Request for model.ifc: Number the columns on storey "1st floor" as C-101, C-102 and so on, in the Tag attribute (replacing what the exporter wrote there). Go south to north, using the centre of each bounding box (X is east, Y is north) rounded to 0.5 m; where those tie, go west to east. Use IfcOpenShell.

First a look at what the model holds.

```python
import ifcopenshell
import ifcopenshell.util.element
import ifcopenshell.util.placement

model = ifcopenshell.open("model.ifc")
print(model.schema)
storey = next(s for s in model.by_type("IfcBuildingStorey") if s.Name == "1st floor")
columns = [e for e in ifcopenshell.util.element.get_decomposition(storey) if e.is_a("IfcColumn")]
for e in sorted(columns, key=lambda e: e.id()):
    origin = ifcopenshell.util.placement.get_local_placement(e.ObjectPlacement)[:3, 3]
    print(e.id(), e.Tag, e.Name, origin.round(2) + 0.0, sep=" | ")
```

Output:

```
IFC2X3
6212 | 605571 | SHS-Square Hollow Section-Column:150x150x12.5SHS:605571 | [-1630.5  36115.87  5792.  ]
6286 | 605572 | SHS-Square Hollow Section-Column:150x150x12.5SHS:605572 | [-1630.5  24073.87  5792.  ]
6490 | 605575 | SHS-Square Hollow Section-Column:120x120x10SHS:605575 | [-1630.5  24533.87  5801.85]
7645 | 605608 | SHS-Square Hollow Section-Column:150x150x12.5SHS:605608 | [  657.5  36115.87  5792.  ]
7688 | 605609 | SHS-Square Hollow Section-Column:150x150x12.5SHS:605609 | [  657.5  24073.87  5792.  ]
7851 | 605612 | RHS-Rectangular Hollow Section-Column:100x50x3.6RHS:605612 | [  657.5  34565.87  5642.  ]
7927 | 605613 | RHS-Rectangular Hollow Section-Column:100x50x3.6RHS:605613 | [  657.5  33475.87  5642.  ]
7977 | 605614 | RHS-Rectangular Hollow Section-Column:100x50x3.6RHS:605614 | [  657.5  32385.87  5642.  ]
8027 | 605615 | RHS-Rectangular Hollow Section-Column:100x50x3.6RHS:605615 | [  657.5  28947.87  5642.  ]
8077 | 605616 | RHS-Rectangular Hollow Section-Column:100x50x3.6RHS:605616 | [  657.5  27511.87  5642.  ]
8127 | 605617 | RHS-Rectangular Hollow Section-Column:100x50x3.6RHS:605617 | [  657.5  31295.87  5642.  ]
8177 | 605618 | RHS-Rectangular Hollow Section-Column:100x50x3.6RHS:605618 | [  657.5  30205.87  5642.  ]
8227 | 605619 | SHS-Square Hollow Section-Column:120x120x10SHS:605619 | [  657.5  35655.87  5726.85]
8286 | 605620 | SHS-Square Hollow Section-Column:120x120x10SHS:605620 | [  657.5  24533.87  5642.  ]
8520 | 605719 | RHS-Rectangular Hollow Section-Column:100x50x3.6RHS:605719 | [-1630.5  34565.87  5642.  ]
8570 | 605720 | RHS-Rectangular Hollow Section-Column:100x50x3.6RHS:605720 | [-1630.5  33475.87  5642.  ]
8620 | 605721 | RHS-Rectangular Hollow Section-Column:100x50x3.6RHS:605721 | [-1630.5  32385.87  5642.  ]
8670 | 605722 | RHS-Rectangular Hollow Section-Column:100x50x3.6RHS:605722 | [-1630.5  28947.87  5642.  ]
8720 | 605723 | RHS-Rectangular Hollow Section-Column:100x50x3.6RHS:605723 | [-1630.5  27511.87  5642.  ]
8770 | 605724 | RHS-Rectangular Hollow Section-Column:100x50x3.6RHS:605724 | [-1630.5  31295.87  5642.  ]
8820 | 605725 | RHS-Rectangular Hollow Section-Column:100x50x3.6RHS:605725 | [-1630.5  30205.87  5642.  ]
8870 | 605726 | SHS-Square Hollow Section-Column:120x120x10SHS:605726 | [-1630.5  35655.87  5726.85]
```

```python
import ifcopenshell
import ifcopenshell.geom
import ifcopenshell.util.element
import ifcopenshell.util.shape

model = ifcopenshell.open("model.ifc")
settings = ifcopenshell.geom.settings()
settings.set("use-world-coords", True)


def centre(element):
    shape = ifcopenshell.geom.create_shape(settings, element)
    return ifcopenshell.util.shape.get_bbox_centroid(shape.geometry)


storey = next(s for s in model.by_type("IfcBuildingStorey") if s.Name == "1st floor")
columns = [e for e in ifcopenshell.util.element.get_decomposition(storey) if e.is_a("IfcColumn")]

# Insertion points can sit at a corner or the storey origin, so sort by the geometry (in metres).
centres = {e: centre(e) for e in columns}
columns.sort(key=lambda e: (round(centres[e][1] / 0.5), centres[e][0]))

for i, e in enumerate(columns, start=1):
    number = f"C-1{i:02d}"
    e.Tag = number
    print(e.id(), number)

model.write("model_updated.ifc")
```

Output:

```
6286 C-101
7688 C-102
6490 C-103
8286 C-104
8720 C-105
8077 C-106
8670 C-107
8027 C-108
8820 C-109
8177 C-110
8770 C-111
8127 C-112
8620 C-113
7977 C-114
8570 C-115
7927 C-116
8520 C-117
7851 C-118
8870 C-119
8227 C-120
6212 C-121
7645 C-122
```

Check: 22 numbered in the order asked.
